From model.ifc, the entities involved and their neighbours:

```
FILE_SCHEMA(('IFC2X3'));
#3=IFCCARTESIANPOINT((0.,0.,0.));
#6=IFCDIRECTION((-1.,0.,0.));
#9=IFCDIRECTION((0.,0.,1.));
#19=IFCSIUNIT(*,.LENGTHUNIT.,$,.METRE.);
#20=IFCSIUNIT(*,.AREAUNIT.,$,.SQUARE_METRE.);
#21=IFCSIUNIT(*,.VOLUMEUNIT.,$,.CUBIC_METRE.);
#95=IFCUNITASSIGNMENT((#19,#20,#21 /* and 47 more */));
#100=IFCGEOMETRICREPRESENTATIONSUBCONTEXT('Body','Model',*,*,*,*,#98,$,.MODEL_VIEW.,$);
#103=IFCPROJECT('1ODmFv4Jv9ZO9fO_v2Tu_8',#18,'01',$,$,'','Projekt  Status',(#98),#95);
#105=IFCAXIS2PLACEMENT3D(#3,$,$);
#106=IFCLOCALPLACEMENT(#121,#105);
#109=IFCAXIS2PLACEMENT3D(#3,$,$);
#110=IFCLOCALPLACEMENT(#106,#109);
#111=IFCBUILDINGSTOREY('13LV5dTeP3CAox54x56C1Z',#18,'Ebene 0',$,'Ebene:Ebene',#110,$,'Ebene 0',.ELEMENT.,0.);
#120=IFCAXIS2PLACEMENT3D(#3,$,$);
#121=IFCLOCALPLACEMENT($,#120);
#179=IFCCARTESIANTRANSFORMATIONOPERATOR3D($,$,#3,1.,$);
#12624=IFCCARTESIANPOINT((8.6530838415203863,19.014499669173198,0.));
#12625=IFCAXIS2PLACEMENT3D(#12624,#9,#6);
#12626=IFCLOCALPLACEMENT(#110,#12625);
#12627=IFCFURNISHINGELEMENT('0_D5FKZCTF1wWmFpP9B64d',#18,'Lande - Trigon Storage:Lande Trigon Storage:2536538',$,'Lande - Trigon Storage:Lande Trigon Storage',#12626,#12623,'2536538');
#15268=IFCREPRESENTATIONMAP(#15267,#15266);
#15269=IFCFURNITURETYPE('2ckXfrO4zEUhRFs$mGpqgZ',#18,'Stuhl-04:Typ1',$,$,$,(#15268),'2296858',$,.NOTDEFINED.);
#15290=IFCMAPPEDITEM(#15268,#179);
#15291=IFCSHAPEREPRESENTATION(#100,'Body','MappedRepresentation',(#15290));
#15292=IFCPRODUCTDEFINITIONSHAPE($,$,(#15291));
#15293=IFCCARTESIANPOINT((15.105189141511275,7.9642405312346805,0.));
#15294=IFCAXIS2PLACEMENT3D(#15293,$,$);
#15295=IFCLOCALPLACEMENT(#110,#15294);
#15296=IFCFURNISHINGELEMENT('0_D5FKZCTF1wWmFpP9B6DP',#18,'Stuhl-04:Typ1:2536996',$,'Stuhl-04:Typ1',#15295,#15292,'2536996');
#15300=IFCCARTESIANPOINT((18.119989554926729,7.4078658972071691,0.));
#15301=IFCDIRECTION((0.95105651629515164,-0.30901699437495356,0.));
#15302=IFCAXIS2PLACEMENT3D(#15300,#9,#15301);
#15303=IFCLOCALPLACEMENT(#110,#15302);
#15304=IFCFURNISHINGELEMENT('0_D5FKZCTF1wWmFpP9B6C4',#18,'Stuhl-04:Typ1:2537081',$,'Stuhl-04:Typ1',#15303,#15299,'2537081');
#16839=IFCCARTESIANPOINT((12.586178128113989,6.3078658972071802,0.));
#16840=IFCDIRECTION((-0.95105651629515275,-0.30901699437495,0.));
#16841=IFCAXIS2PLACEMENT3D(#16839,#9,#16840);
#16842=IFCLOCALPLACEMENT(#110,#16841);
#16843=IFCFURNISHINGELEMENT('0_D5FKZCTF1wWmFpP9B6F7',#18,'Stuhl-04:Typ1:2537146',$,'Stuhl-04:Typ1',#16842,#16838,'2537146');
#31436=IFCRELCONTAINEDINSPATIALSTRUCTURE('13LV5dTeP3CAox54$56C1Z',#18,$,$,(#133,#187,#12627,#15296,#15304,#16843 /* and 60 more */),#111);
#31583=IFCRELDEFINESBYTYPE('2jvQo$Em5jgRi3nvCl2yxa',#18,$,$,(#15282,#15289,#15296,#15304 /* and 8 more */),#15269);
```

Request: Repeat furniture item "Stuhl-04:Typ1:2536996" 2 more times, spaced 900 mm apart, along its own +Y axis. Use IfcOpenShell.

```python
import ifcopenshell
import ifcopenshell.api.geometry
import ifcopenshell.api.root
import ifcopenshell.util.element
import ifcopenshell.util.placement
import ifcopenshell.util.unit

model = ifcopenshell.open("model.ifc")
unit_scale = ifcopenshell.util.unit.calculate_unit_scale(model)

source = model.by_guid("0_D5FKZCTF1wWmFpP9B6DP")
base = ifcopenshell.util.placement.get_local_placement(source.ObjectPlacement)
step = base[:3, 1] * 0.9 / unit_scale

for i in range(1, 3):
    copy = ifcopenshell.api.root.copy_class(model, product=source)
    copy.Representation = ifcopenshell.util.element.copy_deep(
        model, source.Representation, exclude=["IfcGeometricRepresentationContext", "IfcRepresentationMap"]
    )
    copy.Name = "Stuhl-04:Typ1"
    copy.Tag = None
    matrix = base.copy()
    matrix[:3, 3] += i * step
    print("added at", matrix[:3, 3].round(3) + 0.0)
    ifcopenshell.api.geometry.edit_object_placement(model, product=copy, matrix=matrix, is_si=False)

model.write("model_edited.ifc")
```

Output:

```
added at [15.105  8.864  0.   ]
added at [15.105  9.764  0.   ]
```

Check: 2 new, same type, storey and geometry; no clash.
